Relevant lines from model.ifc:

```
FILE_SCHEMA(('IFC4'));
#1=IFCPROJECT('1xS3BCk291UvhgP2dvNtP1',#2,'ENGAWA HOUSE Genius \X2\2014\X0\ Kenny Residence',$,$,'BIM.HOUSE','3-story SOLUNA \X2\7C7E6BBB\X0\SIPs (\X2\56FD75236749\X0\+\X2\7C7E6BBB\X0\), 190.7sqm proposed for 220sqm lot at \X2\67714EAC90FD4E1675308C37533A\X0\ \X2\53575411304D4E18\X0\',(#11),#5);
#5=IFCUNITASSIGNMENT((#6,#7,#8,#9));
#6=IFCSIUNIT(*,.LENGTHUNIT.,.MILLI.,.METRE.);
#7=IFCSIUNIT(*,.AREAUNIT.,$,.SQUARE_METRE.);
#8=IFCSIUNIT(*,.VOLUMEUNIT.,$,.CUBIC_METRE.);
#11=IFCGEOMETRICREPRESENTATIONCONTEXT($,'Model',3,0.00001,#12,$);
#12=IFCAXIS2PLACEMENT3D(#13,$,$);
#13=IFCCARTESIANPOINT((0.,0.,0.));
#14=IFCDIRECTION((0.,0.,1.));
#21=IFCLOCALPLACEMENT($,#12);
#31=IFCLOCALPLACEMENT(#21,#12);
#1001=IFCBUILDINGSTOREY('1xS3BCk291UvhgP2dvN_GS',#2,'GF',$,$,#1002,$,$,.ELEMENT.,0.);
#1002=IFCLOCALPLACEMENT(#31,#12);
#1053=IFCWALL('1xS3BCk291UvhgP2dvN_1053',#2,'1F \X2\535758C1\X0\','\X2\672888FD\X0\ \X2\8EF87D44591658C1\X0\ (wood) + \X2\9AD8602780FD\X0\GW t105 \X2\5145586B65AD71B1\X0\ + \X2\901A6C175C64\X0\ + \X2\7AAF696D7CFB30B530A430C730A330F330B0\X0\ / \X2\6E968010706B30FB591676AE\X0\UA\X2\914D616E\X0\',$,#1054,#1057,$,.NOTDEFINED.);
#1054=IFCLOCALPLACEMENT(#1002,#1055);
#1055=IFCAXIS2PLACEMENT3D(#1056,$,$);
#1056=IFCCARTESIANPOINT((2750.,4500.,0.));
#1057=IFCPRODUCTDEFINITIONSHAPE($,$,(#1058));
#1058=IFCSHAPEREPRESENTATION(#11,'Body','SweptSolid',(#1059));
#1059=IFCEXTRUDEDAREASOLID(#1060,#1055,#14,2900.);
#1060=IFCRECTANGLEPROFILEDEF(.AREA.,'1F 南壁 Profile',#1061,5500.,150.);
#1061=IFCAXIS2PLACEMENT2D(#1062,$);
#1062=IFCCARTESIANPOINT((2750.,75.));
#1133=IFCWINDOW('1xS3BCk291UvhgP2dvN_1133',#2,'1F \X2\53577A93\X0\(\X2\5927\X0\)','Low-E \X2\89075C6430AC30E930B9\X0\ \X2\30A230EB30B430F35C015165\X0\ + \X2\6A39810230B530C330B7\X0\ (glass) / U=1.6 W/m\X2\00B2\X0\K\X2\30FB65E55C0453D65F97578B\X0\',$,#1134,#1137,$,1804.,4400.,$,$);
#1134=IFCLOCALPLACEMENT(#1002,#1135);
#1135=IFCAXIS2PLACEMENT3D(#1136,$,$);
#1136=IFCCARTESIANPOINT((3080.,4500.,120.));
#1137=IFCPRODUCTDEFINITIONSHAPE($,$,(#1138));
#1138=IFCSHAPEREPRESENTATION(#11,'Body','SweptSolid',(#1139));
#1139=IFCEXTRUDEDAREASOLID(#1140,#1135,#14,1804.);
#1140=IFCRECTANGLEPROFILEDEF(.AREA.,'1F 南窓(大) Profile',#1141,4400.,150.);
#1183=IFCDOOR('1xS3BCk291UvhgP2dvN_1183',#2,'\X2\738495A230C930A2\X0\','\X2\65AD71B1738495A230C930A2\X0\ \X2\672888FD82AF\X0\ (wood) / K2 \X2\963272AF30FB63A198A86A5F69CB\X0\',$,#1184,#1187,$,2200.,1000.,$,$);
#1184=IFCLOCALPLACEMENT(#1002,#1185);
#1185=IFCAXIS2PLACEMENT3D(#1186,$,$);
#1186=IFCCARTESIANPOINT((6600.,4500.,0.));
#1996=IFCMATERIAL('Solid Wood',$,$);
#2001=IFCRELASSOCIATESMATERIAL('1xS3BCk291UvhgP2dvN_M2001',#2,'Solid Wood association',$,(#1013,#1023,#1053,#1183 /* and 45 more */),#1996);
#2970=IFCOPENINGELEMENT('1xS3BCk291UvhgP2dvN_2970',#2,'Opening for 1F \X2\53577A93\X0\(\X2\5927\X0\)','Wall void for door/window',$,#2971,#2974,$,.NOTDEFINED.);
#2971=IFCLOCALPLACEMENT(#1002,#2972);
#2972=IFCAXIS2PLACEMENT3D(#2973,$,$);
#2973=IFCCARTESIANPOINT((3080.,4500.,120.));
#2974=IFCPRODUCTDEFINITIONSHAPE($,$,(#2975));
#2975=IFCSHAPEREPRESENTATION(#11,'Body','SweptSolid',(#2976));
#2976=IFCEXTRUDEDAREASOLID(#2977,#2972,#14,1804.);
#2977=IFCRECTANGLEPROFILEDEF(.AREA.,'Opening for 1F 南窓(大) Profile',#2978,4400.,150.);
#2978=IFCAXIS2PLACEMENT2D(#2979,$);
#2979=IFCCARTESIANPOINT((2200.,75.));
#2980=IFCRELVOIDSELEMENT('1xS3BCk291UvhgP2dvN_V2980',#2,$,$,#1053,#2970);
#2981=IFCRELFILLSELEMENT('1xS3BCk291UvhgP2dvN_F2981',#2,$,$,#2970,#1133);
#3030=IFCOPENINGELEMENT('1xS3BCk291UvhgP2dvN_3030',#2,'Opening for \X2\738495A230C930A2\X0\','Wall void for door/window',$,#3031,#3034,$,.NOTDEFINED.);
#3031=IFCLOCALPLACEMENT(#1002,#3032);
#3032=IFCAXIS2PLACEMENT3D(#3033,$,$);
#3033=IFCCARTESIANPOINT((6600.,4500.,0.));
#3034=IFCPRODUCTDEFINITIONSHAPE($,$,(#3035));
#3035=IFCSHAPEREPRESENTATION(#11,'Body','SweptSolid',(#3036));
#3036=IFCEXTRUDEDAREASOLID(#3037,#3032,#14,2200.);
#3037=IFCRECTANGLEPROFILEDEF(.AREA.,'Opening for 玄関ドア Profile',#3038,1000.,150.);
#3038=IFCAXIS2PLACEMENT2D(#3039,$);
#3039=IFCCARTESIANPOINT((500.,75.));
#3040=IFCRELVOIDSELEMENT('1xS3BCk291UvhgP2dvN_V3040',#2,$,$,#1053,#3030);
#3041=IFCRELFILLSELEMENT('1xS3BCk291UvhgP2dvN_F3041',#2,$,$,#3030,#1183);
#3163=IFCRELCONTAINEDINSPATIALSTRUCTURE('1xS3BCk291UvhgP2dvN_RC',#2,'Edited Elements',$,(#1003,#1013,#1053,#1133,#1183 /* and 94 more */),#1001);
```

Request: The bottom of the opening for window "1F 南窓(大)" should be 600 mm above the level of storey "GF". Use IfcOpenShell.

```python
import numpy as np
import ifcopenshell
import ifcopenshell.api.geometry
import ifcopenshell.geom
import ifcopenshell.util.element
import ifcopenshell.util.placement
import ifcopenshell.util.shape
import ifcopenshell.util.unit

model = ifcopenshell.open("model.ifc")
unit_scale = ifcopenshell.util.unit.calculate_unit_scale(model)

window = model.by_id(1133)
opening = window.FillsVoids[0].RelatingOpeningElement
storey = ifcopenshell.util.element.get_container(window, ifc_class="IfcBuildingStorey")
level = ifcopenshell.util.placement.get_local_placement(storey.ObjectPlacement)[2, 3]

# The opening's origin need not be at the sill, so measure its lowest point.
shape = ifcopenshell.geom.create_shape(ifcopenshell.geom.settings(), opening)
bottom = ifcopenshell.util.shape.get_shape_bottom_elevation(shape, shape.geometry) / unit_scale
dz = level + 600.0 - bottom

shift = np.array([0.0, 0.0, dz])
# The window is not placed relative to its opening, so move both.
for product in (opening, window):
    matrix = ifcopenshell.util.placement.get_local_placement(product.ObjectPlacement)
    matrix[:3, 3] += shift
    ifcopenshell.api.geometry.edit_object_placement(model, product=product, matrix=matrix, is_si=False)

print(f"moved by {dz * unit_scale:+.3f} m")

model.write("model_edited.ifc")
```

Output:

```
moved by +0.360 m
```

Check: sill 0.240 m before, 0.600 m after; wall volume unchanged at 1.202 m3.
